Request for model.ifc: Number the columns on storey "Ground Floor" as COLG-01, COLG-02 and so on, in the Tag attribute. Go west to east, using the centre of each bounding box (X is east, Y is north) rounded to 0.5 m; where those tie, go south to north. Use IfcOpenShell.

First a look at what the model holds.

```python
import ifcopenshell
import ifcopenshell.util.element
import ifcopenshell.util.placement

model = ifcopenshell.open("model.ifc")
print(model.schema)
storey = next(s for s in model.by_type("IfcBuildingStorey") if s.Name == "Ground Floor")
columns = [e for e in ifcopenshell.util.element.get_decomposition(storey) if e.is_a("IfcColumn")]
for e in sorted(columns, key=lambda e: e.id()):
    origin = ifcopenshell.util.placement.get_local_placement(e.ObjectPlacement)[:3, 3]
    print(e.id(), e.Tag, e.Name, origin.round(2) + 0.0, sep=" | ")
```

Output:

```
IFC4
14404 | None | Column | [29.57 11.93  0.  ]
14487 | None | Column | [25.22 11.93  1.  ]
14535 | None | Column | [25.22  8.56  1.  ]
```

```python
import ifcopenshell
import ifcopenshell.geom
import ifcopenshell.util.element
import ifcopenshell.util.shape

model = ifcopenshell.open("model.ifc")
settings = ifcopenshell.geom.settings()
settings.set("use-world-coords", True)


def centre(element):
    shape = ifcopenshell.geom.create_shape(settings, element)
    return ifcopenshell.util.shape.get_bbox_centroid(shape.geometry)


storey = next(s for s in model.by_type("IfcBuildingStorey") if s.Name == "Ground Floor")
columns = [e for e in ifcopenshell.util.element.get_decomposition(storey) if e.is_a("IfcColumn")]

# Insertion points can sit at a corner or the storey origin, so sort by the geometry (in metres).
centres = {e: centre(e) for e in columns}
columns.sort(key=lambda e: (round(centres[e][0] / 0.5), centres[e][1]))

for i, e in enumerate(columns, start=1):
    number = f"COLG-{i:02d}"
    e.Tag = number
    print(e.id(), number)

model.write("model_rev.ifc")
```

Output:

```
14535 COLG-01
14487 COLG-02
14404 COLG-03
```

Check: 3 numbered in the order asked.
